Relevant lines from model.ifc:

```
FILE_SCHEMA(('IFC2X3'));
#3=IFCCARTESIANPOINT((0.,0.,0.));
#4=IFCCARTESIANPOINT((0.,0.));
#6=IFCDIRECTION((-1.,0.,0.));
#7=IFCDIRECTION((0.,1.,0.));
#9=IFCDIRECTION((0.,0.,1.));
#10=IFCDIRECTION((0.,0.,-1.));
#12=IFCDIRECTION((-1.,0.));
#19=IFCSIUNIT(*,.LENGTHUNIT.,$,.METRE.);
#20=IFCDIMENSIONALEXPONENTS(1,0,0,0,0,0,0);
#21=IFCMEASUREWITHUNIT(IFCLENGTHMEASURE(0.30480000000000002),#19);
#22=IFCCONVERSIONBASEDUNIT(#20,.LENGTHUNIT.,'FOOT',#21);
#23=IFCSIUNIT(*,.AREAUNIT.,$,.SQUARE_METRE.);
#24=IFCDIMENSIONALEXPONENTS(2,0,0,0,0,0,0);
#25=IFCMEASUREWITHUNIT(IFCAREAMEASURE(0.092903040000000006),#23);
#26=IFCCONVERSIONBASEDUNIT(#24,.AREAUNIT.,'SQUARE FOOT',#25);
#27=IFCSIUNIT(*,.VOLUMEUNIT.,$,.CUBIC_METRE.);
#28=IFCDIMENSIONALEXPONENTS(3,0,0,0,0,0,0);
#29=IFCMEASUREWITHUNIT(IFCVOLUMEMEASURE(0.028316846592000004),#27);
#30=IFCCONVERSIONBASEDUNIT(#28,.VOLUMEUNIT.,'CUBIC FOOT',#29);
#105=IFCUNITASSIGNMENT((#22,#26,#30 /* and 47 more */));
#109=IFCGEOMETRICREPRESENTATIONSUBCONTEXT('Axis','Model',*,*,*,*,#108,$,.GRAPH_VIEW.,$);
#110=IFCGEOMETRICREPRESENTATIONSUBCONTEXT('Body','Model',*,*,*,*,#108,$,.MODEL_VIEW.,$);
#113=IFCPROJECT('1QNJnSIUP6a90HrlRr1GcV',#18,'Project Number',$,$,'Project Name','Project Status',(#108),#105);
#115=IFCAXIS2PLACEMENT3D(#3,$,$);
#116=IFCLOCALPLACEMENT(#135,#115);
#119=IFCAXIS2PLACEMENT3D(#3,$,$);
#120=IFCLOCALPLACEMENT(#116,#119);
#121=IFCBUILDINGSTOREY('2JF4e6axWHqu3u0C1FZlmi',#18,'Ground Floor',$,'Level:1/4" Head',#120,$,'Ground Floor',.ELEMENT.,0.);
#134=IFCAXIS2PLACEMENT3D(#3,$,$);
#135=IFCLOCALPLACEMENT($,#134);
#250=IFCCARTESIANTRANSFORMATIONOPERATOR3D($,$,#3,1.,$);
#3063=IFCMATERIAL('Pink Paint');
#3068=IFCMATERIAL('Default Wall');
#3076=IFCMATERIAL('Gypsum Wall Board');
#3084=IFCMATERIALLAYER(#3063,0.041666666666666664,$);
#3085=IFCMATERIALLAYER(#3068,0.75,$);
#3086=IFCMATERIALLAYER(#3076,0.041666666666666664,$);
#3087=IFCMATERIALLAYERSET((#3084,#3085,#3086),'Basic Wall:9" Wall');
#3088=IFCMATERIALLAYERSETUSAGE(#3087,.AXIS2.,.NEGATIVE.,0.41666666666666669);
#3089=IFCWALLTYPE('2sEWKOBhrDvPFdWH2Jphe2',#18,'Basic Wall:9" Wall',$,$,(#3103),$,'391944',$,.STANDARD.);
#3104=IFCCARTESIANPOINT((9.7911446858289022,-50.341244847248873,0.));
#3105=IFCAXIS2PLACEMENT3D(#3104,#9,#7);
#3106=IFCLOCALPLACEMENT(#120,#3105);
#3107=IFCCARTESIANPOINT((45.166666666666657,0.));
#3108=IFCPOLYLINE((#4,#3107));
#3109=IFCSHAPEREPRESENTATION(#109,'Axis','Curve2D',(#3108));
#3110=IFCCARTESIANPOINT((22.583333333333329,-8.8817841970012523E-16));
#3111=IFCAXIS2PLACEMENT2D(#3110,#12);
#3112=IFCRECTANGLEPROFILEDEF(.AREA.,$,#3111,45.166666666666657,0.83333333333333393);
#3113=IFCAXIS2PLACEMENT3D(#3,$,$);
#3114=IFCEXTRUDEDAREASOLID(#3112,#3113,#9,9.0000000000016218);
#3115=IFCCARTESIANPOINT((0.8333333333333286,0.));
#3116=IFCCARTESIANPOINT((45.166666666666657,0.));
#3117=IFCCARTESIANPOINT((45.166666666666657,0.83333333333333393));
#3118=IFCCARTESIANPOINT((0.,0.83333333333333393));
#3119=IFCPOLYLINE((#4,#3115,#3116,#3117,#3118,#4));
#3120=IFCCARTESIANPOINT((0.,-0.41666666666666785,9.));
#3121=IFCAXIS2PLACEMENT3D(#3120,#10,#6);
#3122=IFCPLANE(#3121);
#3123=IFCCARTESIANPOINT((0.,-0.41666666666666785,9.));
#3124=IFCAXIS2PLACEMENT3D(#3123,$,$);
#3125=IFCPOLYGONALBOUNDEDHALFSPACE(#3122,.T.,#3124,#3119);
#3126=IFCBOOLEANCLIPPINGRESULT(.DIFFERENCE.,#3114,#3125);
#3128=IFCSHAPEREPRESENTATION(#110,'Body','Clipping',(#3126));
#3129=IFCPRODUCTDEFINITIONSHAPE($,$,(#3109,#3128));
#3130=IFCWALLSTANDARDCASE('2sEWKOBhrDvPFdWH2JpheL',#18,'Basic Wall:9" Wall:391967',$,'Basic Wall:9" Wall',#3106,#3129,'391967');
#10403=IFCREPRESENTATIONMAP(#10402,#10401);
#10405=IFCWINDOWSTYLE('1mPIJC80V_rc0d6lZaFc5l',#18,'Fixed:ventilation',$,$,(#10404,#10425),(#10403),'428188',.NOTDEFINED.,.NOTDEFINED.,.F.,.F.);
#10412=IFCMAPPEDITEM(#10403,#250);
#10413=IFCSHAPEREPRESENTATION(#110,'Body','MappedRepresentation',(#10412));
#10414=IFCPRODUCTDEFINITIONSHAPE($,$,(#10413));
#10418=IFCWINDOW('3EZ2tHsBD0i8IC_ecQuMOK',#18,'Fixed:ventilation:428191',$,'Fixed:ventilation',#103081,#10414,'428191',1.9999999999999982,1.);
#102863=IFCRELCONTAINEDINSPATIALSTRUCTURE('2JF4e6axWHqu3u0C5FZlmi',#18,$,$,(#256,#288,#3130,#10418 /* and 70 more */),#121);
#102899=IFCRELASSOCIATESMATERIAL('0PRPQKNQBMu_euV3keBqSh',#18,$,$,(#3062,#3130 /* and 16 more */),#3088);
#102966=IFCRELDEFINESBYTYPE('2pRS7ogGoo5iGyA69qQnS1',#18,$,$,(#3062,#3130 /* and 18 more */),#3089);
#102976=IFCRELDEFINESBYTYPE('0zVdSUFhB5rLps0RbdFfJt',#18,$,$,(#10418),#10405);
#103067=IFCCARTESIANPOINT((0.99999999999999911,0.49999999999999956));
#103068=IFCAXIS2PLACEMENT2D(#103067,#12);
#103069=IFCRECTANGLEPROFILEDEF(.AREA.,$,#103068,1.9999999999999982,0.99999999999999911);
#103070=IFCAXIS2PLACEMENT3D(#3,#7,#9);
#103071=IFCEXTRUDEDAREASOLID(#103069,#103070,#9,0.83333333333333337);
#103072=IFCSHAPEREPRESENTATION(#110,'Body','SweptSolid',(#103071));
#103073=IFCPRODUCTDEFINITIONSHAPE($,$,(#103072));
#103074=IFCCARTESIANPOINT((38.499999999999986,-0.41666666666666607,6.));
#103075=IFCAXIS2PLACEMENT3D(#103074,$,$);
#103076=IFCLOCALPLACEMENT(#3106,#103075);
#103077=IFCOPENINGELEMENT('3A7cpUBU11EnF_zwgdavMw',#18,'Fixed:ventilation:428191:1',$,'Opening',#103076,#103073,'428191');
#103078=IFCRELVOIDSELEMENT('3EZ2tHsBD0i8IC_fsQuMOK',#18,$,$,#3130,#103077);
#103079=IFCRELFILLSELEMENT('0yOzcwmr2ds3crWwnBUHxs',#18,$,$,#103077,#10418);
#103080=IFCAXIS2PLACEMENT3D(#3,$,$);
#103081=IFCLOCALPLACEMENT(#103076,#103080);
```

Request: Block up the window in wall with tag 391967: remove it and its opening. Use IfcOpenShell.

```python
import ifcopenshell
import ifcopenshell.api.feature
import ifcopenshell.api.root
import ifcopenshell.geom
import ifcopenshell.util.shape

model = ifcopenshell.open("model.ifc")
settings = ifcopenshell.geom.settings()


def volume(element):
    """Net volume in cubic metres, openings subtracted."""
    shape = ifcopenshell.geom.create_shape(settings, element)
    return ifcopenshell.util.shape.get_volume(shape.geometry)


window = model.by_guid("3EZ2tHsBD0i8IC_ecQuMOK")
opening = window.FillsVoids[0].RelatingOpeningElement
wall = opening.VoidsElements[0].RelatingBuildingElement
before = volume(wall)

ifcopenshell.api.root.remove_product(model, product=window)
ifcopenshell.api.feature.remove_feature(model, feature=opening)

after = volume(wall)

print(f"wall volume {before:.3f} -> {after:.3f} m3")

model.write("model_updated.ifc")
```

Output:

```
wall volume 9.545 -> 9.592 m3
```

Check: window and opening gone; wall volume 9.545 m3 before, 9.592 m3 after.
